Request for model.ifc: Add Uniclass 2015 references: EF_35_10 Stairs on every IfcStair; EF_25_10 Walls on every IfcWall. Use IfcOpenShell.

First a look at what the model holds.

```python
import ifcopenshell

model = ifcopenshell.open("model.ifc")
print(model.schema)
print("classifications:", [c.Name for c in model.by_type("IfcClassification")])
for ifc_class in ("IfcDoor", "IfcRoof", "IfcStair", "IfcWall", "IfcWindow"):
    print(ifc_class, len(model.by_type(ifc_class)))
```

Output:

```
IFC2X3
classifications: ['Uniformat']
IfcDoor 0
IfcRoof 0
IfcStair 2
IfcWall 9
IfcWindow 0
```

```python
import ifcopenshell
import ifcopenshell.api.classification

model = ifcopenshell.open("model.ifc")

# IFC2X3 requires Source and Edition and has no link from the project to the system.
system = model.create_entity("IfcClassification", Source="NBS", Edition="2015", Name="Uniclass 2015")

codes = {
    "IfcStair": ("EF_35_10", "Stairs"),
    "IfcWall": ("EF_25_10", "Walls"),
}
for ifc_class, (code, name) in codes.items():
    products = model.by_type(ifc_class)
    ifcopenshell.api.classification.add_reference(
        model, products=products, classification=system, identification=code, name=name
    )
    print(code, len(products))

model.write("model_v2.ifc")
```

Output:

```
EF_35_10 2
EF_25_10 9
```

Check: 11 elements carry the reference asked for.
